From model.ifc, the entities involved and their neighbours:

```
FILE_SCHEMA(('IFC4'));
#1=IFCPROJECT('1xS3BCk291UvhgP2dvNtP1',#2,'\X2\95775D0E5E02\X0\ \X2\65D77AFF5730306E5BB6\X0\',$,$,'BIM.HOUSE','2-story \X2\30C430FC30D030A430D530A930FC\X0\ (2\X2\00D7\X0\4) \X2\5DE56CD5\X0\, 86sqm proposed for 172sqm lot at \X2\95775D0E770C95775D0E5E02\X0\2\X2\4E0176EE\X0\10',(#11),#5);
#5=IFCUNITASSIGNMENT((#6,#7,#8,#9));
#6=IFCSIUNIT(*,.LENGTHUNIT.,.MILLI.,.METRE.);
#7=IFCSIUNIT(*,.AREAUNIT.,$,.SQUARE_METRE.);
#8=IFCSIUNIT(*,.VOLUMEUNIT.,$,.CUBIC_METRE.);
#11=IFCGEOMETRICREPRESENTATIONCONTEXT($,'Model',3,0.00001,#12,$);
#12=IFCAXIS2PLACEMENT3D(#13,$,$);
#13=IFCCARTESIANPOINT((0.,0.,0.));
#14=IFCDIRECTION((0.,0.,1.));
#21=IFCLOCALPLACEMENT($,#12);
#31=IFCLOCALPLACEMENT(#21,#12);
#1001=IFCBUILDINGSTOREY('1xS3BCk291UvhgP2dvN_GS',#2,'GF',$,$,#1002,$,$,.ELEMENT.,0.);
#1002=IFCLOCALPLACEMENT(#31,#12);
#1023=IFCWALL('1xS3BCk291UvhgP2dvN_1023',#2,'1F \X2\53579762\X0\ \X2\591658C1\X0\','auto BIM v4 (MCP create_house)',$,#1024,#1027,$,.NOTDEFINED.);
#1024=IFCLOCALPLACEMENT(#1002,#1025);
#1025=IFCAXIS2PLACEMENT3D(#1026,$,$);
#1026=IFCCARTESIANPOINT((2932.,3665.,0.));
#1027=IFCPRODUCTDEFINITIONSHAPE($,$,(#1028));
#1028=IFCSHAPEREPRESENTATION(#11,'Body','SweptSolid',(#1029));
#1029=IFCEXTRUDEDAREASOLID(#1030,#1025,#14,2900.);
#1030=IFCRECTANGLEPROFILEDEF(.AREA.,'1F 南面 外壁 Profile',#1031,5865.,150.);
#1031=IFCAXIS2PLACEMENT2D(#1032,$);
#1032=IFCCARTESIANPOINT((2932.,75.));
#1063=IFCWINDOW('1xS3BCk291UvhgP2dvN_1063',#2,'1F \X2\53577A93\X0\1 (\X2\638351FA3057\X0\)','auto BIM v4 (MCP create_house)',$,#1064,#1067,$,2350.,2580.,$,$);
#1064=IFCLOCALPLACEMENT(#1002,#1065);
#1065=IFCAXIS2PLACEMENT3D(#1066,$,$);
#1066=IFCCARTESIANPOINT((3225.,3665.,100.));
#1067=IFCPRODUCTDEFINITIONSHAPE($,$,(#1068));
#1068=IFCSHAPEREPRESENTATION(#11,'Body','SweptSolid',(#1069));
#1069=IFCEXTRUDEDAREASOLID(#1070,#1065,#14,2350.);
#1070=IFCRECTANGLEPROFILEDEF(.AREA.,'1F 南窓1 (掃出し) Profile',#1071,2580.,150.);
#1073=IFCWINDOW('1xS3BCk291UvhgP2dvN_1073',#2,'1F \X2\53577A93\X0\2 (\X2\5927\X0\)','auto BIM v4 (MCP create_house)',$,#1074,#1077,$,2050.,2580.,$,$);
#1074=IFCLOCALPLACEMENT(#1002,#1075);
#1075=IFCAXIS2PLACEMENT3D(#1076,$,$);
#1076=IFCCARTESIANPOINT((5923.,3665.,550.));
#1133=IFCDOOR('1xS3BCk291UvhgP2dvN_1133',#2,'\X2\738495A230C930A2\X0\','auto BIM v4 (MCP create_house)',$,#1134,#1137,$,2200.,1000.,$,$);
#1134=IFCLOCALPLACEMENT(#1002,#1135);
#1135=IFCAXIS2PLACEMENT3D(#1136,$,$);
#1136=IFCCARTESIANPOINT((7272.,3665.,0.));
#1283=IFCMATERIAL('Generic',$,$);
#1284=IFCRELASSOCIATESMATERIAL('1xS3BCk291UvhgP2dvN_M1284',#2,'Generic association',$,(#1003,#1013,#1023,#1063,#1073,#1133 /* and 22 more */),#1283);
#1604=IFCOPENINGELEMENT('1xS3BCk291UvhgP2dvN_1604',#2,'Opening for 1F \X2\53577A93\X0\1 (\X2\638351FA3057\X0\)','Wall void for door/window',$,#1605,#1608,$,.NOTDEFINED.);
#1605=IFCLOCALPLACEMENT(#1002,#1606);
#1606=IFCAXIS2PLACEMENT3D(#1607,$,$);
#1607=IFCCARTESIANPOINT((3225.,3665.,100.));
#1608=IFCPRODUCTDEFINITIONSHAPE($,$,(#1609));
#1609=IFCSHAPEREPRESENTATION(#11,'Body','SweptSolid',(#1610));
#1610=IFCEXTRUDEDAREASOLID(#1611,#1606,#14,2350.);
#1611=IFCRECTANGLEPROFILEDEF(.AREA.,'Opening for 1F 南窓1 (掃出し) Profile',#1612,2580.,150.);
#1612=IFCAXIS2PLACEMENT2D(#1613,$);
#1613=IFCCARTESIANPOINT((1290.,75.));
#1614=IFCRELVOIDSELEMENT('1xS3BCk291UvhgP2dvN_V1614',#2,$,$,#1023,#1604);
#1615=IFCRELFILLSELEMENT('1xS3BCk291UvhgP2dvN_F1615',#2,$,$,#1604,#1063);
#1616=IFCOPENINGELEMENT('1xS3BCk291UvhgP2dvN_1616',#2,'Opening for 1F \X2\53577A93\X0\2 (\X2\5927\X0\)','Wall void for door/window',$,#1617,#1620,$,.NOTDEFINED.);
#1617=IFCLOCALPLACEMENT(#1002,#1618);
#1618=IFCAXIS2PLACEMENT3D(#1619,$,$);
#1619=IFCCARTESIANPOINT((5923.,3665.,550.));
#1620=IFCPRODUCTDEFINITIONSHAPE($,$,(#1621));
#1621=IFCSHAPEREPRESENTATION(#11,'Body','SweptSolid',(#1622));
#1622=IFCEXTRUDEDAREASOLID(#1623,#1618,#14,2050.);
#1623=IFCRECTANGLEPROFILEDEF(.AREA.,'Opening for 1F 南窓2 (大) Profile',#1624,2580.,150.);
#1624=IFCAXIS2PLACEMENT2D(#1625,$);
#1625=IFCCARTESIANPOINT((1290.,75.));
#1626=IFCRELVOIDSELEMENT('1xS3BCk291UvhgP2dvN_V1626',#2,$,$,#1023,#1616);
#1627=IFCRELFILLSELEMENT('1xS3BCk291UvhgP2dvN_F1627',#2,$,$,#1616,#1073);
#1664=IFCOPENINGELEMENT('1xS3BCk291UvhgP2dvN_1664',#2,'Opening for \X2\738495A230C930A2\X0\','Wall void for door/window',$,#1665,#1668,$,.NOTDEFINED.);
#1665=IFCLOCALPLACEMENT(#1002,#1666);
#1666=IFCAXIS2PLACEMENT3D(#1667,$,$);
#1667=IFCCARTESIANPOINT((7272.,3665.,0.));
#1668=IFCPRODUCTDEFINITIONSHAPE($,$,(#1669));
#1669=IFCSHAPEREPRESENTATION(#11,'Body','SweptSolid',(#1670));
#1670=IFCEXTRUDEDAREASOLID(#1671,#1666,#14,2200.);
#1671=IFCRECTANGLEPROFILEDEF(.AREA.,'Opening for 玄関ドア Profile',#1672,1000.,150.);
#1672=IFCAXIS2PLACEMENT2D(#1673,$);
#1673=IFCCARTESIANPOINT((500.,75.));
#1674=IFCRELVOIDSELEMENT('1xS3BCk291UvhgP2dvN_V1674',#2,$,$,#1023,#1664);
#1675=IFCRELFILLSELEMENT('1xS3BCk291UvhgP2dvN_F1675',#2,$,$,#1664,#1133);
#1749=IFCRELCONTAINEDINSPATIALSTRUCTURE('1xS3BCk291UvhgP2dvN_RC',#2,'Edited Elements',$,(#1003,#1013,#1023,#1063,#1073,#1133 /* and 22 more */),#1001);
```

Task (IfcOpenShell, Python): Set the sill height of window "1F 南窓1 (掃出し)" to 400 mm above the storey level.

```python
import numpy as np
import ifcopenshell
import ifcopenshell.api.geometry
import ifcopenshell.geom
import ifcopenshell.util.element
import ifcopenshell.util.placement
import ifcopenshell.util.shape
import ifcopenshell.util.unit

model = ifcopenshell.open("model.ifc")
unit_scale = ifcopenshell.util.unit.calculate_unit_scale(model)

window = model.by_guid("1xS3BCk291UvhgP2dvN_1063")
opening = window.FillsVoids[0].RelatingOpeningElement
storey = ifcopenshell.util.element.get_container(window, ifc_class="IfcBuildingStorey")
level = ifcopenshell.util.placement.get_local_placement(storey.ObjectPlacement)[2, 3]

# The opening's origin need not be at the sill, so measure its lowest point.
shape = ifcopenshell.geom.create_shape(ifcopenshell.geom.settings(), opening)
bottom = ifcopenshell.util.shape.get_shape_bottom_elevation(shape, shape.geometry) / unit_scale
dz = level + 0.4 / unit_scale - bottom

shift = np.array([0.0, 0.0, dz])
# The window is not placed relative to its opening, so move both.
for product in (opening, window):
    matrix = ifcopenshell.util.placement.get_local_placement(product.ObjectPlacement)
    matrix[:3, 3] += shift
    ifcopenshell.api.geometry.edit_object_placement(model, product=product, matrix=matrix, is_si=False)

print(f"moved by {dz * unit_scale:+.3f} m")

model.write("model-out.ifc")
```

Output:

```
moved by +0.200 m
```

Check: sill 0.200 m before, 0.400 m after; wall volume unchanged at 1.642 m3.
